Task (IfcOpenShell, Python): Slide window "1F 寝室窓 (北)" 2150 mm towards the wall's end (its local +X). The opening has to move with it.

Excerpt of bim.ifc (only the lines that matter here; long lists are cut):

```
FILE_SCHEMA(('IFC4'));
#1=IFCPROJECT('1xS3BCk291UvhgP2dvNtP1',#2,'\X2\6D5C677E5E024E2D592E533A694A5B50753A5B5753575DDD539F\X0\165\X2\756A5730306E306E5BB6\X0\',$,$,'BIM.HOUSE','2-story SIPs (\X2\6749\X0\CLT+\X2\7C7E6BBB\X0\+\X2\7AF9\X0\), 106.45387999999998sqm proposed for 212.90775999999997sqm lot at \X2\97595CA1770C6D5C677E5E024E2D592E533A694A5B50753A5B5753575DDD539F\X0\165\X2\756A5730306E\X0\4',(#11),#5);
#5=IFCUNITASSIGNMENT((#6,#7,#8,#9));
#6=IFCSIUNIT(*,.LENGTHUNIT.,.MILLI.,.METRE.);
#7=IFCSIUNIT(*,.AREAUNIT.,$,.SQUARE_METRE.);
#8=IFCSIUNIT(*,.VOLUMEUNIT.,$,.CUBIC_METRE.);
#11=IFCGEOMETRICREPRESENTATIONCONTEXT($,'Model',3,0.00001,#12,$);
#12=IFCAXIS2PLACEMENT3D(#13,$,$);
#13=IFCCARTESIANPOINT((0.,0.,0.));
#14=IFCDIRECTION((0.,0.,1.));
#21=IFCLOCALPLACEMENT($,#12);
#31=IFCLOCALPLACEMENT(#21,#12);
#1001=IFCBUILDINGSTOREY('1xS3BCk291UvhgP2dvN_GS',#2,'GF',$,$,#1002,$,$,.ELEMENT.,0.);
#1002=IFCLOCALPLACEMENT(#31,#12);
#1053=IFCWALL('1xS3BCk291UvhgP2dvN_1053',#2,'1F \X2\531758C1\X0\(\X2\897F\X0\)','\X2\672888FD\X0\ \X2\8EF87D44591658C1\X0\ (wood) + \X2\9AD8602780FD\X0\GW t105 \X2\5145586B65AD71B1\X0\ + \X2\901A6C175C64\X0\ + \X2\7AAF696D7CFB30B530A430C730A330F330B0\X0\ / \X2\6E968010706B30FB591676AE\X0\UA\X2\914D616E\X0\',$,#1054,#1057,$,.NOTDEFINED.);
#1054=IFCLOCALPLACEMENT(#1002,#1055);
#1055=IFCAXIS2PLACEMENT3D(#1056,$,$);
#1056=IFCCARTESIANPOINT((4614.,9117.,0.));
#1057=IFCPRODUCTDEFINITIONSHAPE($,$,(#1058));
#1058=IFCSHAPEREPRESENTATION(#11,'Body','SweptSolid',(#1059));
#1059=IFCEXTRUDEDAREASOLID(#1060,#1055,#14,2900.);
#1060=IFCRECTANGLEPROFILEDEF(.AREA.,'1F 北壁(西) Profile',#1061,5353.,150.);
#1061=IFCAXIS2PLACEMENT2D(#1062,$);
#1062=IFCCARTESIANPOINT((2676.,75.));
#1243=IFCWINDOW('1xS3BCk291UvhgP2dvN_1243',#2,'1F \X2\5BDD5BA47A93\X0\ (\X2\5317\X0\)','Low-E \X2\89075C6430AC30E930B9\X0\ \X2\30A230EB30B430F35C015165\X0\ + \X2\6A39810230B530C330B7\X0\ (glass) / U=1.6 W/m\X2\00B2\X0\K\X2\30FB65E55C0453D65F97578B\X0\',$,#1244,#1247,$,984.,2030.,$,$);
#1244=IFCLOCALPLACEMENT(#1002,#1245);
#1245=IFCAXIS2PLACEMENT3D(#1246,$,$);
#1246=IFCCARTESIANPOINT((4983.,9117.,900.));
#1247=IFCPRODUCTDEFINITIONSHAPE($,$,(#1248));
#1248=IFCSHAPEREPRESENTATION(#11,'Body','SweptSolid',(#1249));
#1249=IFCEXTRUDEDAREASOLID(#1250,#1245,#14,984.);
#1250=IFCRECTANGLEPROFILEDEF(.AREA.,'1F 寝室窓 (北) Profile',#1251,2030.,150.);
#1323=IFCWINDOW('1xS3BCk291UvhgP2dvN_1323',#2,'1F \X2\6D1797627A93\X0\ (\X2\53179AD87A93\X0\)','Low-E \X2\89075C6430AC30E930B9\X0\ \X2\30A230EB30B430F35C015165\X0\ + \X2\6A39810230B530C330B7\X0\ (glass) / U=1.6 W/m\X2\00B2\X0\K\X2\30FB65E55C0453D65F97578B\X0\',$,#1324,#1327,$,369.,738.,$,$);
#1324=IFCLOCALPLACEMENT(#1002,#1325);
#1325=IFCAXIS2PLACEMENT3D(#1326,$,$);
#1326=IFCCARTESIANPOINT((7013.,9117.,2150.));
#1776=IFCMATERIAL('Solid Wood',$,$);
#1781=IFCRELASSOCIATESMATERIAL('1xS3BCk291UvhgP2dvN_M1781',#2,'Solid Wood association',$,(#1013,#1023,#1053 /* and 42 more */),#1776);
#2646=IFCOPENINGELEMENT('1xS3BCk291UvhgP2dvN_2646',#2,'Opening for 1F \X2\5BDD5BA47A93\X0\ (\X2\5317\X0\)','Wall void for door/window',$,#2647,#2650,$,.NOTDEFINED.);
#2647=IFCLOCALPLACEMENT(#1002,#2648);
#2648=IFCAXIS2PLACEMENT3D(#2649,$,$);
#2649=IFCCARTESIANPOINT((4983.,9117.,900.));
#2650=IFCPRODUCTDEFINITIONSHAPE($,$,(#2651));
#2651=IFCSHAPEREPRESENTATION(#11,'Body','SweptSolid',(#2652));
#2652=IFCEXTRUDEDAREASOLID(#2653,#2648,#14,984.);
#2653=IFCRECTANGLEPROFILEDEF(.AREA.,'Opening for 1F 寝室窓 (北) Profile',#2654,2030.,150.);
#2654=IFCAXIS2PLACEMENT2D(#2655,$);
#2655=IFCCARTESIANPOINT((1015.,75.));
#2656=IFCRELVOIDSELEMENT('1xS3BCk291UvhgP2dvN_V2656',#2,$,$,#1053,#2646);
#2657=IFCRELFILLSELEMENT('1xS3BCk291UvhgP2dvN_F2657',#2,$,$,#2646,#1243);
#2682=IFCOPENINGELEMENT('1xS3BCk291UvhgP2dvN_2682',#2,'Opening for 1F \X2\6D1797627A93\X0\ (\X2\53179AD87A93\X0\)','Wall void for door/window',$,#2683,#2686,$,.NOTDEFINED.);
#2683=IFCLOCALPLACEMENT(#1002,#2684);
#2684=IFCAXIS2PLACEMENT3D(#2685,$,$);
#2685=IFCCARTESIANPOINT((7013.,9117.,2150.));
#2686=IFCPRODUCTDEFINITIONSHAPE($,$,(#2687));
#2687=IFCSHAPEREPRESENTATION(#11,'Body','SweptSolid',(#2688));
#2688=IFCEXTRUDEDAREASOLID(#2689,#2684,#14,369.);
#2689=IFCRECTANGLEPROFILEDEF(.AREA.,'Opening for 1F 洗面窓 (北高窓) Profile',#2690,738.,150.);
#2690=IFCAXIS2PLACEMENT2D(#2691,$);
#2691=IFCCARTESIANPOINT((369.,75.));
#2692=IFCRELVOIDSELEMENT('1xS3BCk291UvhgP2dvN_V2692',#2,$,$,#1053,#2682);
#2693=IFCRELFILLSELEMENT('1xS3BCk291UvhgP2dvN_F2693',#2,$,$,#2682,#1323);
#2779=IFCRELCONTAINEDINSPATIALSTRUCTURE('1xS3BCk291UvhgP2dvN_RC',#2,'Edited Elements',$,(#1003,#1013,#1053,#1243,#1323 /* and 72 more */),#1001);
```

```python
import ifcopenshell
import ifcopenshell.api.geometry
import ifcopenshell.util.placement

model = ifcopenshell.open("bim.ifc")

window = model.by_guid("1xS3BCk291UvhgP2dvN_1243")
opening = window.FillsVoids[0].RelatingOpeningElement
wall = opening.VoidsElements[0].RelatingBuildingElement

wall_matrix = ifcopenshell.util.placement.get_local_placement(wall.ObjectPlacement)
shift = wall_matrix[:3, 0] * 2150.0
before = ifcopenshell.util.placement.get_local_placement(window.ObjectPlacement)[:3, 3].copy()

# The window is not placed relative to its opening, so move both.
for product in (opening, window):
    matrix = ifcopenshell.util.placement.get_local_placement(product.ObjectPlacement)
    matrix[:3, 3] += shift
    ifcopenshell.api.geometry.edit_object_placement(model, product=product, matrix=matrix, is_si=False)

after = ifcopenshell.util.placement.get_local_placement(window.ObjectPlacement)[:3, 3]
print("window moved by", (after - before).round(3) + 0.0)

model.write("bim_rev.ifc")
```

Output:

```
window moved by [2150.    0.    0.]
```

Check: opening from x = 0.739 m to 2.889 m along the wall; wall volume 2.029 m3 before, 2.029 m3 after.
